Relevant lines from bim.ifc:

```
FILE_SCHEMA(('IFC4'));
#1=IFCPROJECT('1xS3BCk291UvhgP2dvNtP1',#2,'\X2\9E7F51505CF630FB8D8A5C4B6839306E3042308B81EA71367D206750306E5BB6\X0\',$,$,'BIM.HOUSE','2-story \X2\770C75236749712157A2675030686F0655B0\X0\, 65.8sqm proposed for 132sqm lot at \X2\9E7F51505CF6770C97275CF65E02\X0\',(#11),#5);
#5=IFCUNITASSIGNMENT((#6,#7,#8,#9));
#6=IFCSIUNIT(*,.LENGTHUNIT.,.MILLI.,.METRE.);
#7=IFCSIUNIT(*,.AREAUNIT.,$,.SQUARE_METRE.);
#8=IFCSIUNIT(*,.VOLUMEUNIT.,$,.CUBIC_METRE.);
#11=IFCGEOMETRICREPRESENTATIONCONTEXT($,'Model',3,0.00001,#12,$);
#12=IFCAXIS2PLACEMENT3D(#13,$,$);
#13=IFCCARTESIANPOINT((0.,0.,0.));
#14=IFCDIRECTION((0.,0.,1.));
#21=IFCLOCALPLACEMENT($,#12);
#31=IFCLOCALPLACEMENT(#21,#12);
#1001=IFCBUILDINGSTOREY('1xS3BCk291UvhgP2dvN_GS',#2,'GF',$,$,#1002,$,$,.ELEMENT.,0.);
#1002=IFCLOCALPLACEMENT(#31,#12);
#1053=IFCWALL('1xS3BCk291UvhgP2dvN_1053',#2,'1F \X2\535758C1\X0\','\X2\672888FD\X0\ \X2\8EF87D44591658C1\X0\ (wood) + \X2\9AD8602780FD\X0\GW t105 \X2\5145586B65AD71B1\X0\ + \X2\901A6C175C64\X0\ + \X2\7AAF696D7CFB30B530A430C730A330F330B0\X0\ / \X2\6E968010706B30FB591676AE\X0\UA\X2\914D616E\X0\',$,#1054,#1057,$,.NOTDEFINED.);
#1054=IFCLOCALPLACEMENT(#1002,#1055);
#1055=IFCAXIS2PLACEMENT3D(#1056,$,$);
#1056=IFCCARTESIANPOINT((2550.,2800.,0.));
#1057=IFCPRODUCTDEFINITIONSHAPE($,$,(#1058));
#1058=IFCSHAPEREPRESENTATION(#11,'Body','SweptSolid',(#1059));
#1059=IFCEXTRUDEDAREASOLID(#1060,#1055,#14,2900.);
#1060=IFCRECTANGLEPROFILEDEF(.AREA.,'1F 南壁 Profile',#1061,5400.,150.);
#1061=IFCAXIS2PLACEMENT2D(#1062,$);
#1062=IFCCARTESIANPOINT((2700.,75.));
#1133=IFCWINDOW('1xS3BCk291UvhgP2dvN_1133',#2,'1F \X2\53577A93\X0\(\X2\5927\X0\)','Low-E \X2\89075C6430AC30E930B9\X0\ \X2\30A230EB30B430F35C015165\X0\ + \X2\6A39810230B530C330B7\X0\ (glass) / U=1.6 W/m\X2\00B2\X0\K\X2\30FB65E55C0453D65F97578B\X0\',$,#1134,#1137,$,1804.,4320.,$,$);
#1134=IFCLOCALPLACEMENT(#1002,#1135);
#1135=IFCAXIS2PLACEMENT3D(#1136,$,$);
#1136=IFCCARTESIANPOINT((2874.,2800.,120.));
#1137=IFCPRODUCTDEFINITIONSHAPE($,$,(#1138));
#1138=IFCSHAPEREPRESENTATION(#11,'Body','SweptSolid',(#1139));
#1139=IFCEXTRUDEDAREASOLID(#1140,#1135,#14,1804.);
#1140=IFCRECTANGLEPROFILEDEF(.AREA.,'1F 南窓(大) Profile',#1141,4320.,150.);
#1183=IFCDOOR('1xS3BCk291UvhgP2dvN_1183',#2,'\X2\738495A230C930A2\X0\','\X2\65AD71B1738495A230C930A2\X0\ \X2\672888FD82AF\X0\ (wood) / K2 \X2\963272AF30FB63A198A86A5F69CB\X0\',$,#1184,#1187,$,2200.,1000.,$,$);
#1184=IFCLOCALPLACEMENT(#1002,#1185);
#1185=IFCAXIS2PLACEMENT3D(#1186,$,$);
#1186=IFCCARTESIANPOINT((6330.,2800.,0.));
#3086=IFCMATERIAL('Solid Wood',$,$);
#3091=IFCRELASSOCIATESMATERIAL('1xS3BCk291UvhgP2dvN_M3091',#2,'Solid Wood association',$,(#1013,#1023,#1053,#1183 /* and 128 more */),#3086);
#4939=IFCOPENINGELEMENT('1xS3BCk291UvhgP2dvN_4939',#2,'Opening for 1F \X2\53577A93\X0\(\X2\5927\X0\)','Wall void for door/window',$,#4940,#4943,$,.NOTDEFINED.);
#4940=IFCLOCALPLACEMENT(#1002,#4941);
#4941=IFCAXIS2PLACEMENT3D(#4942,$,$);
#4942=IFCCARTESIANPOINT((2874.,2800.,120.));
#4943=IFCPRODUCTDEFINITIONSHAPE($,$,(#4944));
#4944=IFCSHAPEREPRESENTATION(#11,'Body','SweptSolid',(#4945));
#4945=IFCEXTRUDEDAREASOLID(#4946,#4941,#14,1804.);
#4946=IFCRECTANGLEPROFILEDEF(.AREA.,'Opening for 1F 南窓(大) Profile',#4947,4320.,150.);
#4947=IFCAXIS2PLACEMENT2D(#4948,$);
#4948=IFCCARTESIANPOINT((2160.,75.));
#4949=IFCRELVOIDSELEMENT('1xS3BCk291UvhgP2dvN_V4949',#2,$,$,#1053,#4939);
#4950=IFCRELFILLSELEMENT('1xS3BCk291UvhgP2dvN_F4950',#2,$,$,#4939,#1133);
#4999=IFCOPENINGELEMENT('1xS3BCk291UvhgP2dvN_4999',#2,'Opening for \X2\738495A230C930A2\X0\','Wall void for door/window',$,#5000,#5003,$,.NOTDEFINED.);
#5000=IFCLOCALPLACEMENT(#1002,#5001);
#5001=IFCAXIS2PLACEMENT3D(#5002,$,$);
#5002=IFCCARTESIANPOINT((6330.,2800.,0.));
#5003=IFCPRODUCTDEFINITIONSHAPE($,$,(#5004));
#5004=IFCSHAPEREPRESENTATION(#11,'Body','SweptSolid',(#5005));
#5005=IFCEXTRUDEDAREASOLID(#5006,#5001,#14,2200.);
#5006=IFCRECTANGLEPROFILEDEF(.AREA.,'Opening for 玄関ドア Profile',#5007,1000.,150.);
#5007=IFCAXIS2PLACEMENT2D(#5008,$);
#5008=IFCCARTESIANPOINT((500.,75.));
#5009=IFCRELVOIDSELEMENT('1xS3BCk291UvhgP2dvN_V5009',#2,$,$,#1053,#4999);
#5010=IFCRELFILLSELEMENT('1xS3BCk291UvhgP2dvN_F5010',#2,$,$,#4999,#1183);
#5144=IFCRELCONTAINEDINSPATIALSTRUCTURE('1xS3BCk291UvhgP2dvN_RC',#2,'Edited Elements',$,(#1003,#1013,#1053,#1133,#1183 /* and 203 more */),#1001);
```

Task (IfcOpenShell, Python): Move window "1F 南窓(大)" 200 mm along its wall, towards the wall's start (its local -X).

```python
import ifcopenshell
import ifcopenshell.api.geometry
import ifcopenshell.util.placement
import ifcopenshell.util.unit

model = ifcopenshell.open("bim.ifc")
unit_scale = ifcopenshell.util.unit.calculate_unit_scale(model)

window = model.by_guid("1xS3BCk291UvhgP2dvN_1133")
opening = window.FillsVoids[0].RelatingOpeningElement
wall = opening.VoidsElements[0].RelatingBuildingElement

wall_matrix = ifcopenshell.util.placement.get_local_placement(wall.ObjectPlacement)
shift = wall_matrix[:3, 0] * -0.2 / unit_scale
before = ifcopenshell.util.placement.get_local_placement(window.ObjectPlacement)[:3, 3].copy()

# The window is not placed relative to its opening, so move both.
for product in (opening, window):
    matrix = ifcopenshell.util.placement.get_local_placement(product.ObjectPlacement)
    matrix[:3, 3] += shift
    ifcopenshell.api.geometry.edit_object_placement(model, product=product, matrix=matrix, is_si=False)

after = ifcopenshell.util.placement.get_local_placement(window.ObjectPlacement)[:3, 3]
print("window moved by", (after - before).round(3) + 0.0)

model.write("bim_v2.ifc")
```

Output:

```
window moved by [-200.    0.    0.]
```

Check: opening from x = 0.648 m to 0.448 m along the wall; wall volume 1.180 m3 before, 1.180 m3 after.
